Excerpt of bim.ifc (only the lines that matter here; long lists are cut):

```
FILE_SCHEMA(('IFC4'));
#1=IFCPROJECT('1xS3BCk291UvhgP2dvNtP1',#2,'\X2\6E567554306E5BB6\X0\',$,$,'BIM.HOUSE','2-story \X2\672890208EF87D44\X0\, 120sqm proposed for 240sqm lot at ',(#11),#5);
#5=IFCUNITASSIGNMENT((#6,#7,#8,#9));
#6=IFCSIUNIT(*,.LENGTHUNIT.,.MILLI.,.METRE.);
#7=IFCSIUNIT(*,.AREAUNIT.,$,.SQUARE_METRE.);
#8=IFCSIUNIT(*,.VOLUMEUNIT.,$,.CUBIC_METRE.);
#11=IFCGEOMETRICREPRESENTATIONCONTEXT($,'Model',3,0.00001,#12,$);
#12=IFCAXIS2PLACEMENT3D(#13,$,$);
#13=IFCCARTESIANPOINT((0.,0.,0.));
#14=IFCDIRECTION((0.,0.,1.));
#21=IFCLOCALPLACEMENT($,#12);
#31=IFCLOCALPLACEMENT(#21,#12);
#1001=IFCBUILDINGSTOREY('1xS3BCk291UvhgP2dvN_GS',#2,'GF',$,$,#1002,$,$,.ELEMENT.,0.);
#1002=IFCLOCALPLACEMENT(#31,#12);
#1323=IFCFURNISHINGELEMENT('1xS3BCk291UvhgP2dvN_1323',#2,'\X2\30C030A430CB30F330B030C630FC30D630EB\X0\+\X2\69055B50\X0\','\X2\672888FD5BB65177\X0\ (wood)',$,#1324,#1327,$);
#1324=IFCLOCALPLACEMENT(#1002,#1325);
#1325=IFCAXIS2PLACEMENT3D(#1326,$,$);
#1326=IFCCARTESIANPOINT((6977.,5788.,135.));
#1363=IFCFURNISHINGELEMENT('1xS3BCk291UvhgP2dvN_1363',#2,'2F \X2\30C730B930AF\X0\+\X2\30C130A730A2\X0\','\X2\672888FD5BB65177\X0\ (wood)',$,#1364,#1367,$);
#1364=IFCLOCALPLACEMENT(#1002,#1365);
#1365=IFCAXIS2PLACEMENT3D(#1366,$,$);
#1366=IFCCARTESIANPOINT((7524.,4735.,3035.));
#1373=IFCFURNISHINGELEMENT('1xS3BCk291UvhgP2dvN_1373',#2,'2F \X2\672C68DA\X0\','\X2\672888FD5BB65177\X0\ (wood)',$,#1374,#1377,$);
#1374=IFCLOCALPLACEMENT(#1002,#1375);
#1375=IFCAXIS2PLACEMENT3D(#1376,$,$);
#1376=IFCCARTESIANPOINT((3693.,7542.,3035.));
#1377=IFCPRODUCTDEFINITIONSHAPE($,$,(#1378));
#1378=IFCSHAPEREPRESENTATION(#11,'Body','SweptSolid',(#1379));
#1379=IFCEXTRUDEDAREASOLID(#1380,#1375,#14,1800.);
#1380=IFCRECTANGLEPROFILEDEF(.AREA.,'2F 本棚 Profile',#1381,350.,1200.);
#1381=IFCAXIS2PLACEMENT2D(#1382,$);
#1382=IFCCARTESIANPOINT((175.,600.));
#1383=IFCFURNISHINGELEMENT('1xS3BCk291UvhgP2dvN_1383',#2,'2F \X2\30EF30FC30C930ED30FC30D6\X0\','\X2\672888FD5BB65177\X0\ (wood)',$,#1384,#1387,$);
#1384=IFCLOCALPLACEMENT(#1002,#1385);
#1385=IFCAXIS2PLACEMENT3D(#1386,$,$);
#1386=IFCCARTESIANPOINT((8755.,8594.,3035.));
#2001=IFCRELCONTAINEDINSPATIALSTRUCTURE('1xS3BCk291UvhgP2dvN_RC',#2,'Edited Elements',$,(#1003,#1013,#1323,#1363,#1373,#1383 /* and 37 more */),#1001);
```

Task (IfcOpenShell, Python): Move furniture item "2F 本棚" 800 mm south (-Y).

```python
import ifcopenshell
import ifcopenshell.api.geometry
import ifcopenshell.util.placement
import ifcopenshell.util.unit

model = ifcopenshell.open("bim.ifc")
unit_scale = ifcopenshell.util.unit.calculate_unit_scale(model)

item = model.by_id(1373)
matrix = ifcopenshell.util.placement.get_local_placement(item.ObjectPlacement)
matrix[1, 3] -= 0.8 / unit_scale
ifcopenshell.api.geometry.edit_object_placement(model, product=item, matrix=matrix, is_si=False)

print(ifcopenshell.util.placement.get_local_placement(item.ObjectPlacement).round(3) + 0.0)

model.write("bim-out.ifc")
```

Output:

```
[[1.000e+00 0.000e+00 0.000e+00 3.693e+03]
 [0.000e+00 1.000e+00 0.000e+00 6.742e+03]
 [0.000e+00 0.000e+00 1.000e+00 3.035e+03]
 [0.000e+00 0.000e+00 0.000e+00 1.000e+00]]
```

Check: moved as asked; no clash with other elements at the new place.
